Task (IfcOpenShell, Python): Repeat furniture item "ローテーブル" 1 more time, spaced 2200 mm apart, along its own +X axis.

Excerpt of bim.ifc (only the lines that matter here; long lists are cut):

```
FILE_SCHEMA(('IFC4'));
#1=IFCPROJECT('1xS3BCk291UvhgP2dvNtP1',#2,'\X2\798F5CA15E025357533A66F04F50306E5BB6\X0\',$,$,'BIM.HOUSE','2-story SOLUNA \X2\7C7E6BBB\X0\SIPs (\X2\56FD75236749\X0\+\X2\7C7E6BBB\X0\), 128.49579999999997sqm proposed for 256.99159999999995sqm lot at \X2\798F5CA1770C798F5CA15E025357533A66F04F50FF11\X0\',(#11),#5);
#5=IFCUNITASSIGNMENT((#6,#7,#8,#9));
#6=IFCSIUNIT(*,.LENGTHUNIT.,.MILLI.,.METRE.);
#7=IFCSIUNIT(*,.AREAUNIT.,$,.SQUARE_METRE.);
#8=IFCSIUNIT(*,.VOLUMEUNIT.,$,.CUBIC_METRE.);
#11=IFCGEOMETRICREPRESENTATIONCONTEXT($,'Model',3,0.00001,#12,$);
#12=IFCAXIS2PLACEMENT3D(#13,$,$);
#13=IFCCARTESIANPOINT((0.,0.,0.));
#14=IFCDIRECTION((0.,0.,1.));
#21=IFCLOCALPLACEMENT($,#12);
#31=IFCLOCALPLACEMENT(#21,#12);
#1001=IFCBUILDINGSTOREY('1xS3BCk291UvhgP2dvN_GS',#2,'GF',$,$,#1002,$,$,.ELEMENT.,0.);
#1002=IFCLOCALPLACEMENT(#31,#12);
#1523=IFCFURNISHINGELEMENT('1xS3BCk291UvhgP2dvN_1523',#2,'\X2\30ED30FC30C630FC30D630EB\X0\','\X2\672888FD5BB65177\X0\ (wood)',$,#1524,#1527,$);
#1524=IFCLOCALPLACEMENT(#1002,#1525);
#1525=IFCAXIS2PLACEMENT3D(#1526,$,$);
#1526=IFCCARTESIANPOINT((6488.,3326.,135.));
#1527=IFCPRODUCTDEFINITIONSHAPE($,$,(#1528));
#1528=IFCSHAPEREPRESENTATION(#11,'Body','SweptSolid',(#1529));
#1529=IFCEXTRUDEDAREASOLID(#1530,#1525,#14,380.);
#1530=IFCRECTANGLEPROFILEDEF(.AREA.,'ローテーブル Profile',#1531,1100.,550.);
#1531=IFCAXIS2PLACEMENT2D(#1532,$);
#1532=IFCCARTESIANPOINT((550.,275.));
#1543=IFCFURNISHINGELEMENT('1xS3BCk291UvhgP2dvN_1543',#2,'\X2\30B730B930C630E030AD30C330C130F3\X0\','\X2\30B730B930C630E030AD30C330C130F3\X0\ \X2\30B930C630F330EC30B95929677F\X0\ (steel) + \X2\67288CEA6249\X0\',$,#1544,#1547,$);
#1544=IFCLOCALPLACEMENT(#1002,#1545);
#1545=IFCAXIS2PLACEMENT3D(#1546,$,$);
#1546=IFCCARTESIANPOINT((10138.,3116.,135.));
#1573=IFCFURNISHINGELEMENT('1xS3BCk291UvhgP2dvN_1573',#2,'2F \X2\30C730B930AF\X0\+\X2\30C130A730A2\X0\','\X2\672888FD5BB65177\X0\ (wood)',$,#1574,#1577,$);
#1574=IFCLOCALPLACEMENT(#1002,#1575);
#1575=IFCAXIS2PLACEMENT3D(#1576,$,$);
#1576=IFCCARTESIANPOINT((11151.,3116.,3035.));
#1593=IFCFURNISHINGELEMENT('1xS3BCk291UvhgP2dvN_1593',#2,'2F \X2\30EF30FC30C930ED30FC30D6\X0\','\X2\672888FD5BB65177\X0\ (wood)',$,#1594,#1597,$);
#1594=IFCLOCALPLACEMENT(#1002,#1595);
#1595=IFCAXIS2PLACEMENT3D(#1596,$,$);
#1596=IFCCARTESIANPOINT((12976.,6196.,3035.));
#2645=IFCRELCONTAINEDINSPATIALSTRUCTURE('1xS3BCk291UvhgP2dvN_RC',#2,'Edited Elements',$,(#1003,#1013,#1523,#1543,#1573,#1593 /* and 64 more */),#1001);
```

```python
import ifcopenshell
import ifcopenshell.api.geometry
import ifcopenshell.api.root
import ifcopenshell.util.element
import ifcopenshell.util.placement
import ifcopenshell.util.unit

model = ifcopenshell.open("bim.ifc")
unit_scale = ifcopenshell.util.unit.calculate_unit_scale(model)


def reuse_history(source, copy):
    """copy_class also copies each property set's owner history, people and application; keep the originals."""
    for rel in copy.IsDefinedBy:
        if rel.is_a("IfcRelDefinesByProperties") and (history := rel.RelatingPropertyDefinition.OwnerHistory):
            rel.RelatingPropertyDefinition.OwnerHistory = source.OwnerHistory
            ifcopenshell.util.element.remove_deep2(model, history)


source = model.by_guid("1xS3BCk291UvhgP2dvN_1523")
base = ifcopenshell.util.placement.get_local_placement(source.ObjectPlacement)
step = base[:3, 0] * 2.2 / unit_scale

for i in range(1, 2):
    copy = ifcopenshell.api.root.copy_class(model, product=source)
    copy.Representation = ifcopenshell.util.element.copy_deep(
        model, source.Representation, exclude=["IfcGeometricRepresentationContext", "IfcRepresentationMap"]
    )
    reuse_history(source, copy)
    matrix = base.copy()
    matrix[:3, 3] += i * step
    print("added at", matrix[:3, 3].round(3) + 0.0)
    ifcopenshell.api.geometry.edit_object_placement(model, product=copy, matrix=matrix, is_si=False)

model.write("bim_updated.ifc")
```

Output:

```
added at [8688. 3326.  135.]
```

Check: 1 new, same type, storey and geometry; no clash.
